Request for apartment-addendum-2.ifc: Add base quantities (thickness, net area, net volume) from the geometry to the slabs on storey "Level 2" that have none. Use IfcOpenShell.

First a look at what the model holds.

```python
import ifcopenshell
import ifcopenshell.util.element
import ifcopenshell.util.unit

model = ifcopenshell.open("apartment-addendum-2.ifc")
print(model.schema)
for unit_type in ("LENGTHUNIT", "AREAUNIT", "VOLUMEUNIT"):
    print(unit_type, ifcopenshell.util.unit.calculate_unit_scale(model, unit_type))
storey = next(s for s in model.by_type("IfcBuildingStorey") if s.Name == "Level 2")
slabs = [e for e in ifcopenshell.util.element.get_decomposition(storey) if e.is_a("IfcSlab")]
for e in sorted(slabs, key=lambda e: e.id()):
    print(e.id(), e.is_a(), e.Name, list(ifcopenshell.util.element.get_psets(e, qtos_only=True)), sep=" | ")
```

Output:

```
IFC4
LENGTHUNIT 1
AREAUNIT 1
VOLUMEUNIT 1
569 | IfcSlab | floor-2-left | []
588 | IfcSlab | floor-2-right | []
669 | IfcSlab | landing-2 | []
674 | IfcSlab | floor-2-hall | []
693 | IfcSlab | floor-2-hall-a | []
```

```python
import ifcopenshell
import ifcopenshell.api.pset
import ifcopenshell.geom
import ifcopenshell.util.element
import ifcopenshell.util.shape
import ifcopenshell.util.unit

model = ifcopenshell.open("apartment-addendum-2.ifc")
unit_scale = ifcopenshell.util.unit.calculate_unit_scale(model)
area_scale = ifcopenshell.util.unit.calculate_unit_scale(model, "AREAUNIT")
volume_scale = ifcopenshell.util.unit.calculate_unit_scale(model, "VOLUMEUNIT")
settings = ifcopenshell.geom.settings()

storey = next(s for s in model.by_type("IfcBuildingStorey") if s.Name == "Level 2")
slabs = [e for e in ifcopenshell.util.element.get_decomposition(storey) if e.is_a("IfcSlab")]

for e in sorted(slabs, key=lambda e: e.id()):
    if ifcopenshell.util.element.get_psets(e, qtos_only=True, should_inherit=False):
        continue
    # Geometry comes back in metres, in the element's own axes.
    shape = ifcopenshell.geom.create_shape(settings, e)
    values = {
        "Width": ifcopenshell.util.shape.get_z(shape.geometry) / unit_scale,
        "NetArea": ifcopenshell.util.shape.get_footprint_area(shape.geometry) / area_scale,
        "NetVolume": ifcopenshell.util.shape.get_volume(shape.geometry) / volume_scale,
    }
    qto = ifcopenshell.api.pset.add_qto(model, product=e, name="Qto_SlabBaseQuantities")
    ifcopenshell.api.pset.edit_qto(model, qto=qto, properties=values)
    print(e.id(), {k: round(v, 3) for k, v in values.items()})

model.write("apartment-addendum-2_updated.ifc")
```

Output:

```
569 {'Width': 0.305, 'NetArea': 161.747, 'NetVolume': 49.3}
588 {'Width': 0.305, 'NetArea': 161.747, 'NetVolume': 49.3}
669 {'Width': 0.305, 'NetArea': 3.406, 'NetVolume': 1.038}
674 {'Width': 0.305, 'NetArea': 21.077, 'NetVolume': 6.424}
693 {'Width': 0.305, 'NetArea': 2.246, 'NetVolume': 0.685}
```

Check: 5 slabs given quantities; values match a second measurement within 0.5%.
